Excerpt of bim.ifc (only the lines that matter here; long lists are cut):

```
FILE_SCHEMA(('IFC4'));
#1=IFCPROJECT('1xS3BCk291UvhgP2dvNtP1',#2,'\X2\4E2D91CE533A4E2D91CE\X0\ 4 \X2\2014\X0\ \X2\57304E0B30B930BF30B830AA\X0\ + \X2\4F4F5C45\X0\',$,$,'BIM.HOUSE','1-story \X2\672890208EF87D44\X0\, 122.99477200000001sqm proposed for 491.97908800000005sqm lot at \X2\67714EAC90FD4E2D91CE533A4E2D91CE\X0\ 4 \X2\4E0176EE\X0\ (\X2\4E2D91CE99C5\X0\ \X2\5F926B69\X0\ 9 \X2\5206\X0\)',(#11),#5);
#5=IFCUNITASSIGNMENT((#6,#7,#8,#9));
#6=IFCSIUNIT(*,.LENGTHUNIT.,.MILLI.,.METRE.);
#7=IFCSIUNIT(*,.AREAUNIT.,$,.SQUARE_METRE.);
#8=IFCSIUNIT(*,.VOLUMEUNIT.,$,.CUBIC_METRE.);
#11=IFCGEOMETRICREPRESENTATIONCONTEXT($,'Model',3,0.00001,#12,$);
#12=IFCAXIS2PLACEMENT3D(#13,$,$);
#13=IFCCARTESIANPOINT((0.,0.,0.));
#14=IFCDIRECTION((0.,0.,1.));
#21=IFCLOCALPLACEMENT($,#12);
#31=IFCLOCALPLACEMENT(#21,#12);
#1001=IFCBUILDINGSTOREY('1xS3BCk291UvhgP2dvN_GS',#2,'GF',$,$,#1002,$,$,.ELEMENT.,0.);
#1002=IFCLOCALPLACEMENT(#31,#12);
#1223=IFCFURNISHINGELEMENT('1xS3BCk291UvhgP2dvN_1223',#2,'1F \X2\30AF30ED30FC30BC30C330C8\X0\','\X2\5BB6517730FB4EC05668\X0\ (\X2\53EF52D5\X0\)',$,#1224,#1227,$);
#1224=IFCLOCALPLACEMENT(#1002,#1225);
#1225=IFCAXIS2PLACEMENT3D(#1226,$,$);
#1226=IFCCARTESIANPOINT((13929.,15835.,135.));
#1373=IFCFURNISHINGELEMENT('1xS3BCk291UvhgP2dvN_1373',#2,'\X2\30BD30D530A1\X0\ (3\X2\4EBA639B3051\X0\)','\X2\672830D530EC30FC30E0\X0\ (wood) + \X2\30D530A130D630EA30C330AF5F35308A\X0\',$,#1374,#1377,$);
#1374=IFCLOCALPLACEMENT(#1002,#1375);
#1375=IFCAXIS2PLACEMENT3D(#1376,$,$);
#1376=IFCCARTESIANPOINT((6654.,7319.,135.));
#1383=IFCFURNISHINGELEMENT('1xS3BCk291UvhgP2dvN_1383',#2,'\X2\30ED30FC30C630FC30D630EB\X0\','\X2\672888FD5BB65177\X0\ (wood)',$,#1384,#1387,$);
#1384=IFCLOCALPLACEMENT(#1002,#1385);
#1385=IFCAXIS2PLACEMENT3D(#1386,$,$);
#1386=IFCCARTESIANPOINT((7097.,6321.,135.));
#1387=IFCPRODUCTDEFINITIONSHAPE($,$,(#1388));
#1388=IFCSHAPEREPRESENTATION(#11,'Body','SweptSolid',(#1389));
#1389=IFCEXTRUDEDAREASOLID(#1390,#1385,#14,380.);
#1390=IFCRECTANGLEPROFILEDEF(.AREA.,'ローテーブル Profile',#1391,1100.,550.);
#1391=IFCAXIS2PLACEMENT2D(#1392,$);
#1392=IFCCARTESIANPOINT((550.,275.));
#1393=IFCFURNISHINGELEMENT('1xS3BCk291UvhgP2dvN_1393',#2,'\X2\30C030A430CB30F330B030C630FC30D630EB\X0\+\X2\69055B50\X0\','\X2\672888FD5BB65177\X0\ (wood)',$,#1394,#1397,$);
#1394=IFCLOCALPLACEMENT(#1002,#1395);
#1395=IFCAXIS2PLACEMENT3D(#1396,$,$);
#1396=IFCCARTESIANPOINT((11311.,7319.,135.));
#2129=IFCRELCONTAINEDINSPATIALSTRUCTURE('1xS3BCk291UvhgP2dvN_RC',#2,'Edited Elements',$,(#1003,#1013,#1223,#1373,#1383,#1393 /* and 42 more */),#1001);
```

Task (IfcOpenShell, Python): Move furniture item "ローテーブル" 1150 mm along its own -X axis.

```python
import ifcopenshell
import ifcopenshell.api.geometry
import ifcopenshell.util.placement

model = ifcopenshell.open("bim.ifc")

item = model.by_guid("1xS3BCk291UvhgP2dvN_1383")
matrix = ifcopenshell.util.placement.get_local_placement(item.ObjectPlacement)
matrix[:3, 3] -= matrix[:3, 0] * 1150.0
ifcopenshell.api.geometry.edit_object_placement(model, product=item, matrix=matrix, is_si=False)

print(ifcopenshell.util.placement.get_local_placement(item.ObjectPlacement).round(3) + 0.0)

model.write("bim_rev.ifc")
```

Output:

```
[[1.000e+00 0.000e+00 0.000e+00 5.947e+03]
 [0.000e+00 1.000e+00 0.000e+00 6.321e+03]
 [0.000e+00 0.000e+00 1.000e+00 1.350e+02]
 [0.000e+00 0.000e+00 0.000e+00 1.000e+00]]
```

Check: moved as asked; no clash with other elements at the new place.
